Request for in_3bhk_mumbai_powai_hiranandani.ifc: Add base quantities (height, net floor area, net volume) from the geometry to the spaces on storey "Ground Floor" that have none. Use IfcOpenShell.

First a look at what the model holds.

```python
import ifcopenshell
import ifcopenshell.util.element
import ifcopenshell.util.unit

model = ifcopenshell.open("in_3bhk_mumbai_powai_hiranandani.ifc")
print(model.schema)
for unit_type in ("LENGTHUNIT", "AREAUNIT", "VOLUMEUNIT"):
    print(unit_type, ifcopenshell.util.unit.calculate_unit_scale(model, unit_type))
storey = next(s for s in model.by_type("IfcBuildingStorey") if s.Name == "Ground Floor")
spaces = [e for e in ifcopenshell.util.element.get_decomposition(storey) if e.is_a("IfcSpace")]
for e in sorted(spaces, key=lambda e: e.id()):
    print(e.id(), e.is_a(), e.Name, list(ifcopenshell.util.element.get_psets(e, qtos_only=True)), sep=" | ")
```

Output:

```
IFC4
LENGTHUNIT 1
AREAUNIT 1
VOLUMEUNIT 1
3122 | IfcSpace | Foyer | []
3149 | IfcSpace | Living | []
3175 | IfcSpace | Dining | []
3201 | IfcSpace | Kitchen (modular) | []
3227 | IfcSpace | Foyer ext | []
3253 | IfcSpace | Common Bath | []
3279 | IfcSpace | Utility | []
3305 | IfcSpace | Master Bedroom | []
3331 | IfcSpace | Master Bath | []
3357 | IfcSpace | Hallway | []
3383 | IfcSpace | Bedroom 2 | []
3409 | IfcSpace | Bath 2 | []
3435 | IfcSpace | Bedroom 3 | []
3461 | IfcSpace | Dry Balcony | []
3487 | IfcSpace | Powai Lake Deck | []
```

```python
import ifcopenshell
import ifcopenshell.api.pset
import ifcopenshell.geom
import ifcopenshell.util.element
import ifcopenshell.util.shape
import ifcopenshell.util.unit

model = ifcopenshell.open("in_3bhk_mumbai_powai_hiranandani.ifc")
unit_scale = ifcopenshell.util.unit.calculate_unit_scale(model)
area_scale = ifcopenshell.util.unit.calculate_unit_scale(model, "AREAUNIT")
volume_scale = ifcopenshell.util.unit.calculate_unit_scale(model, "VOLUMEUNIT")
settings = ifcopenshell.geom.settings()

storey = next(s for s in model.by_type("IfcBuildingStorey") if s.Name == "Ground Floor")
spaces = [e for e in ifcopenshell.util.element.get_decomposition(storey) if e.is_a("IfcSpace")]

for e in sorted(spaces, key=lambda e: e.id()):
    if ifcopenshell.util.element.get_psets(e, qtos_only=True, should_inherit=False):
        continue
    # Geometry comes back in metres, in the element's own axes.
    shape = ifcopenshell.geom.create_shape(settings, e)
    values = {
        "Height": ifcopenshell.util.shape.get_z(shape.geometry) / unit_scale,
        "NetFloorArea": ifcopenshell.util.shape.get_footprint_area(shape.geometry) / area_scale,
        "NetVolume": ifcopenshell.util.shape.get_volume(shape.geometry) / volume_scale,
    }
    qto = ifcopenshell.api.pset.add_qto(model, product=e, name="Qto_SpaceBaseQuantities")
    ifcopenshell.api.pset.edit_qto(model, qto=qto, properties=values)
    print(e.id(), {k: round(v, 3) for k, v in values.items()})

model.write("in_3bhk_mumbai_powai_hiranandani_edited.ifc")
```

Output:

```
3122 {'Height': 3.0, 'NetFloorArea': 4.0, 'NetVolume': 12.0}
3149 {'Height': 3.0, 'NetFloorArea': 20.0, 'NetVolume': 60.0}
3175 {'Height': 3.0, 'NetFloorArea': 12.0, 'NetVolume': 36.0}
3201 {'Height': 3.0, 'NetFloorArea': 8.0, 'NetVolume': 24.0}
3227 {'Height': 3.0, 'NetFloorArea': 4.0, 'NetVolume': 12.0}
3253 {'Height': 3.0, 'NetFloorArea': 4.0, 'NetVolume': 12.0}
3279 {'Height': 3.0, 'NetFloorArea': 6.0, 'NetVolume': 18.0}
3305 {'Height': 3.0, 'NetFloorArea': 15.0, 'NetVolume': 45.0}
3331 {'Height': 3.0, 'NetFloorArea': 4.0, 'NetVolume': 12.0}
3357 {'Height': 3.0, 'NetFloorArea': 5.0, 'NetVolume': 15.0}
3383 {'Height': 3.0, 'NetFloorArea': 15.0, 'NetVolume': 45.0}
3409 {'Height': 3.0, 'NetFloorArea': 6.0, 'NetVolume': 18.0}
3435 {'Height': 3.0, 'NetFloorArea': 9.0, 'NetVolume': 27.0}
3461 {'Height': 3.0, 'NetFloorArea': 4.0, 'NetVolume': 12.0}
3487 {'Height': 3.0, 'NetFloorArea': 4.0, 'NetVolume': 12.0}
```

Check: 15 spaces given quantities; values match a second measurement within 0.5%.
